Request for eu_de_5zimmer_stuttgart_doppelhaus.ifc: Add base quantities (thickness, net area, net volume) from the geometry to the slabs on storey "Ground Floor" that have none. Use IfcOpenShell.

First a look at what the model holds.

```python
import ifcopenshell
import ifcopenshell.util.element
import ifcopenshell.util.unit

model = ifcopenshell.open("eu_de_5zimmer_stuttgart_doppelhaus.ifc")
print(model.schema)
for unit_type in ("LENGTHUNIT", "AREAUNIT", "VOLUMEUNIT"):
    print(unit_type, ifcopenshell.util.unit.calculate_unit_scale(model, unit_type))
storey = next(s for s in model.by_type("IfcBuildingStorey") if s.Name == "Ground Floor")
slabs = [e for e in ifcopenshell.util.element.get_decomposition(storey) if e.is_a("IfcSlab")]
for e in sorted(slabs, key=lambda e: e.id()):
    print(e.id(), e.is_a(), e.Name, list(ifcopenshell.util.element.get_psets(e, qtos_only=True)), sep=" | ")
```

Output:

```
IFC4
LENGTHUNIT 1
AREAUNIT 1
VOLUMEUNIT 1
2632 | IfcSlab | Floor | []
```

```python
import ifcopenshell
import ifcopenshell.api.pset
import ifcopenshell.geom
import ifcopenshell.util.element
import ifcopenshell.util.shape
import ifcopenshell.util.unit

model = ifcopenshell.open("eu_de_5zimmer_stuttgart_doppelhaus.ifc")
unit_scale = ifcopenshell.util.unit.calculate_unit_scale(model)
area_scale = ifcopenshell.util.unit.calculate_unit_scale(model, "AREAUNIT")
volume_scale = ifcopenshell.util.unit.calculate_unit_scale(model, "VOLUMEUNIT")
settings = ifcopenshell.geom.settings()

storey = next(s for s in model.by_type("IfcBuildingStorey") if s.Name == "Ground Floor")
slabs = [e for e in ifcopenshell.util.element.get_decomposition(storey) if e.is_a("IfcSlab")]

for e in sorted(slabs, key=lambda e: e.id()):
    if ifcopenshell.util.element.get_psets(e, qtos_only=True, should_inherit=False):
        continue
    # Geometry comes back in metres, in the element's own axes.
    shape = ifcopenshell.geom.create_shape(settings, e)
    values = {
        "Width": ifcopenshell.util.shape.get_z(shape.geometry) / unit_scale,
        "NetArea": ifcopenshell.util.shape.get_footprint_area(shape.geometry) / area_scale,
        "NetVolume": ifcopenshell.util.shape.get_volume(shape.geometry) / volume_scale,
    }
    qto = ifcopenshell.api.pset.add_qto(model, product=e, name="Qto_SlabBaseQuantities")
    ifcopenshell.api.pset.edit_qto(model, qto=qto, properties=values)
    print(e.id(), {k: round(v, 3) for k, v in values.items()})

model.write("eu_de_5zimmer_stuttgart_doppelhaus_rev.ifc")
```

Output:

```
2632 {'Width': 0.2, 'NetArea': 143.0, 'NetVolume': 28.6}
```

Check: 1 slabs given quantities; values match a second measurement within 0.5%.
